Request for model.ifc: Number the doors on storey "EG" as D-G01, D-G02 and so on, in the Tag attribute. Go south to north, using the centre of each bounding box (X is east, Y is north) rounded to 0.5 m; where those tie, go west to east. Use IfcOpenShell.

First a look at what the model holds.

```python
import ifcopenshell
import ifcopenshell.util.element
import ifcopenshell.util.placement

model = ifcopenshell.open("model.ifc")
print(model.schema)
storey = next(s for s in model.by_type("IfcBuildingStorey") if s.Name == "EG")
doors = [e for e in ifcopenshell.util.element.get_decomposition(storey) if e.is_a("IfcDoor")]
for e in sorted(doors, key=lambda e: e.id()):
    origin = ifcopenshell.util.placement.get_local_placement(e.ObjectPlacement)[:3, 3]
    print(e.id(), e.Tag, e.Name, origin.round(2) + 0.0, sep=" | ")
```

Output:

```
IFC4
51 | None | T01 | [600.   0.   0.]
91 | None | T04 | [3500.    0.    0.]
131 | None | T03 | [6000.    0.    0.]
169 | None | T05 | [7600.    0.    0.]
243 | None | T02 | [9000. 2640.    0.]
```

```python
import ifcopenshell
import ifcopenshell.geom
import ifcopenshell.util.element
import ifcopenshell.util.shape

model = ifcopenshell.open("model.ifc")
settings = ifcopenshell.geom.settings()
settings.set("use-world-coords", True)


def centre(element):
    shape = ifcopenshell.geom.create_shape(settings, element)
    return ifcopenshell.util.shape.get_bbox_centroid(shape.geometry)


storey = next(s for s in model.by_type("IfcBuildingStorey") if s.Name == "EG")
doors = [e for e in ifcopenshell.util.element.get_decomposition(storey) if e.is_a("IfcDoor")]

# Insertion points can sit at a corner or the storey origin, so sort by the geometry (in metres).
centres = {e: centre(e) for e in doors}
doors.sort(key=lambda e: (round(centres[e][1] / 0.5), centres[e][0]))

for i, e in enumerate(doors, start=1):
    number = f"D-G{i:02d}"
    e.Tag = number
    print(e.id(), number)

model.write("model-out.ifc")
```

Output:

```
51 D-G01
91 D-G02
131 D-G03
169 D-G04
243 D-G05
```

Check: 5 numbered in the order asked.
